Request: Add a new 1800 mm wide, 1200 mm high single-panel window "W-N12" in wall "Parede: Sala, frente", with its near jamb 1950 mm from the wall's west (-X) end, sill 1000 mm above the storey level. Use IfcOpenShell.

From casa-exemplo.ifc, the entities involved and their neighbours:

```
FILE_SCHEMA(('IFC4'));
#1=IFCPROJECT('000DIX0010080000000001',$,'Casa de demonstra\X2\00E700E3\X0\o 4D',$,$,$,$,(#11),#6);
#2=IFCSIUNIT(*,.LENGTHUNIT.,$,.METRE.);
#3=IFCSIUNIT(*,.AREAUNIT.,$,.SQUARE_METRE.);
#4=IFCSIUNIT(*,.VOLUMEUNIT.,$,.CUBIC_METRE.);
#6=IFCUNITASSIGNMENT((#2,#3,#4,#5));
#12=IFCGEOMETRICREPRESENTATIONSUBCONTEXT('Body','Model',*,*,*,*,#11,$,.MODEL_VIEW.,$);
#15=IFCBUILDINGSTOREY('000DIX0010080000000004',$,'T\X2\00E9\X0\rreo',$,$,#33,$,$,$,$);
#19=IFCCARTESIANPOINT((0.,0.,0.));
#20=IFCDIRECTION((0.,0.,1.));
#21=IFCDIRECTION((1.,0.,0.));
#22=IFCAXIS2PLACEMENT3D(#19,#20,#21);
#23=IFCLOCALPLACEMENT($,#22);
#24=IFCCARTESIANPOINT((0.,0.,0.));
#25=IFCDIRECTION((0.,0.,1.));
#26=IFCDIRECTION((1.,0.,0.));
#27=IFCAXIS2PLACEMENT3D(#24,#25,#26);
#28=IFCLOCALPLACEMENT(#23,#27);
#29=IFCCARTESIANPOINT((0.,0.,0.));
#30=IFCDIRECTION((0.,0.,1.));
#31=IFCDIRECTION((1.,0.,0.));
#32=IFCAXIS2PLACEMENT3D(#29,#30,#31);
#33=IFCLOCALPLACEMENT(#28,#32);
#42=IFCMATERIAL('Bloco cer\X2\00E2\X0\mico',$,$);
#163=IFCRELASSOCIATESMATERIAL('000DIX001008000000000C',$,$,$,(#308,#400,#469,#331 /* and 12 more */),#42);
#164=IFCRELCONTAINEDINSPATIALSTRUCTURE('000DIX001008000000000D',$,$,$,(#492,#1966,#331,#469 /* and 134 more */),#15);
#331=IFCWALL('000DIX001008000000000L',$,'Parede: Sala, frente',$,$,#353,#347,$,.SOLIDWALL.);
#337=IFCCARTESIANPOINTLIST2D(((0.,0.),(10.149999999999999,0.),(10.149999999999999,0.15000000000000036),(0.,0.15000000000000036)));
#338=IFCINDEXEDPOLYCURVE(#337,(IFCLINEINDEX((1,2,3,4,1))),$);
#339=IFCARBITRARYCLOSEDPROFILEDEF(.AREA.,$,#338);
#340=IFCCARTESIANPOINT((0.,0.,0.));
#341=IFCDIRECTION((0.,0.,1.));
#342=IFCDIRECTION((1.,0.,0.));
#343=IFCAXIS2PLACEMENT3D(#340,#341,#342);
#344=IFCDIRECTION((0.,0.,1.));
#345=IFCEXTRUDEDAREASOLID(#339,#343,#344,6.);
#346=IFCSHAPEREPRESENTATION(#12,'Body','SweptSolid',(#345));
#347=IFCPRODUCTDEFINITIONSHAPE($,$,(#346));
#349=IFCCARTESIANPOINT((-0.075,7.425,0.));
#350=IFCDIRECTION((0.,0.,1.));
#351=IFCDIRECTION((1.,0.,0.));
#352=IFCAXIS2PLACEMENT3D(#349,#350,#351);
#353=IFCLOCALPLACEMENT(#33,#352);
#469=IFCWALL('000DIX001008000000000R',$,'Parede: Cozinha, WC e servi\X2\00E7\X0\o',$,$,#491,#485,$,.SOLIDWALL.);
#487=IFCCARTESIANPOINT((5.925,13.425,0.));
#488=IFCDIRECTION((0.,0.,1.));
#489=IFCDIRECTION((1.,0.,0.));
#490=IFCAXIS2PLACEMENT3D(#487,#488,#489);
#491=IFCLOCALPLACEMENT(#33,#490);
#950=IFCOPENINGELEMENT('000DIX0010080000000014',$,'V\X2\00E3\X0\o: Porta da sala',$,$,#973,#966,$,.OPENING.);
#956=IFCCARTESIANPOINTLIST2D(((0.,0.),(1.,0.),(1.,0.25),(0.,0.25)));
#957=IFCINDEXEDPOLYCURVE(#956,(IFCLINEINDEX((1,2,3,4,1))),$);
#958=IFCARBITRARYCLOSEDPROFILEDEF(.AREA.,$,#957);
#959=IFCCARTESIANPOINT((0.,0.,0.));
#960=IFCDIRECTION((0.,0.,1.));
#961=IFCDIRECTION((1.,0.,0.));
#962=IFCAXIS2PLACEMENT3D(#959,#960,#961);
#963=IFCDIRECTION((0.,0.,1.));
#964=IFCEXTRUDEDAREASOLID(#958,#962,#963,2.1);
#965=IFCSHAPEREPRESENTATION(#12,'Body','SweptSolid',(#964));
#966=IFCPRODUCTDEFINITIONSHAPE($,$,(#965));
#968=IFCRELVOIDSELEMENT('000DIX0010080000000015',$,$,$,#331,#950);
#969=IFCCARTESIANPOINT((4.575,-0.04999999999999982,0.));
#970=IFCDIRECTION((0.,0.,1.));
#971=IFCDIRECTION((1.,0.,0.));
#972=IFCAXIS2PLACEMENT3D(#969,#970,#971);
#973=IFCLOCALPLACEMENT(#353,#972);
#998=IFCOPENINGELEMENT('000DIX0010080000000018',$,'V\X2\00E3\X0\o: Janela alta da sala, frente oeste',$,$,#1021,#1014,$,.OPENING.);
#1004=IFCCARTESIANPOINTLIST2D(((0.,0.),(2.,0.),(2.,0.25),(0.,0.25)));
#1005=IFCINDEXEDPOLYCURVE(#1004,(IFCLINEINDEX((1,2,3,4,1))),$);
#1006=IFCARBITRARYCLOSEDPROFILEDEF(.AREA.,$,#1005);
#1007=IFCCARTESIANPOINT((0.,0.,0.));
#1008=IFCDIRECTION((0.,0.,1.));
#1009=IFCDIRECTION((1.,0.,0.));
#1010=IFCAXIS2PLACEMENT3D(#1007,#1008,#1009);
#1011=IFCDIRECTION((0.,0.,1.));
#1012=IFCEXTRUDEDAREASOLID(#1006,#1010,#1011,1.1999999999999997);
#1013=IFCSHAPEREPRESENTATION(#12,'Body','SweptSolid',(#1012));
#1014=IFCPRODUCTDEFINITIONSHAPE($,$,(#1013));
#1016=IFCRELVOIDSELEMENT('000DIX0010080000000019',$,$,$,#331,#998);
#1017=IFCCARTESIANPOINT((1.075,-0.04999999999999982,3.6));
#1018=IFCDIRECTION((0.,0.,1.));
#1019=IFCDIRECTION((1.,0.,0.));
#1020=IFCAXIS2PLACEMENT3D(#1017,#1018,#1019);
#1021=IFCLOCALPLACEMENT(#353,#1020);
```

```python
import numpy as np
import ifcopenshell
import ifcopenshell.api.feature
import ifcopenshell.api.geometry
import ifcopenshell.api.root
import ifcopenshell.api.spatial
import ifcopenshell.geom
import ifcopenshell.util.element
import ifcopenshell.util.placement
import ifcopenshell.util.representation
import ifcopenshell.util.shape
import ifcopenshell.util.unit

model = ifcopenshell.open("casa-exemplo.ifc")
unit_scale = ifcopenshell.util.unit.calculate_unit_scale(model)
settings = ifcopenshell.geom.settings()


def volume(element):
    """Net volume in cubic metres, openings subtracted."""
    shape = ifcopenshell.geom.create_shape(settings, element)
    return ifcopenshell.util.shape.get_volume(shape.geometry)


wall = model.by_guid("000DIX001008000000000L")
storey = ifcopenshell.util.element.get_container(wall, ifc_class="IfcBuildingStorey")
context = ifcopenshell.util.representation.get_context(model, "Model", "Body", "MODEL_VIEW")
before = volume(wall)

width, height, from_end, sill = 1.8, 1.2, 1.95, 1  # metres

# The wall runs along its own X axis, and the end named is its -X end.
wall_shape = ifcopenshell.geom.create_shape(settings, wall)
x, y, z = ifcopenshell.util.shape.get_vertices(wall_shape.geometry).T
start = x.min() + from_end
face, thickness = float(y.min()), float(y.max() - y.min())
wall_matrix = ifcopenshell.util.placement.get_local_placement(wall.ObjectPlacement)
level = ifcopenshell.util.placement.get_local_placement(storey.ObjectPlacement)[2, 3]


def in_wall(x, y):
    """Placement at x, y metres in the wall's axes, at sill height."""
    matrix = wall_matrix.copy()
    matrix[:, 3] = wall_matrix @ np.array([x / unit_scale, y / unit_scale, 0.0, 1.0])
    matrix[2, 3] = level + sill / unit_scale
    return matrix


# Opening: a box that overshoots both wall faces by 50 mm.
opening = ifcopenshell.api.root.create_entity(model, ifc_class="IfcOpeningElement", predefined_type="OPENING")
box = ifcopenshell.api.geometry.add_wall_representation(
    model, context=context, length=width, height=height, thickness=thickness + 0.1
)
ifcopenshell.api.geometry.assign_representation(model, product=opening, representation=box)
ifcopenshell.api.geometry.edit_object_placement(model, product=opening, matrix=in_wall(start, face - 0.05), is_si=False)
ifcopenshell.api.feature.add_feature(model, feature=opening, element=wall)

window = ifcopenshell.api.root.create_entity(model, ifc_class="IfcWindow", name="W-N12", predefined_type="WINDOW")
window.OverallWidth, window.OverallHeight = width / unit_scale, height / unit_scale
window.PartitioningType = "SINGLE_PANEL"
body = ifcopenshell.api.geometry.add_window_representation(
    model,
    context=context,
    overall_width=window.OverallWidth,
    overall_height=window.OverallHeight,
    partition_type="SINGLE_PANEL",
)
ifcopenshell.api.geometry.assign_representation(model, product=window, representation=body)
ifcopenshell.api.spatial.assign_container(model, products=[window], relating_structure=storey)
ifcopenshell.api.feature.add_filling(model, opening=opening, element=window)

# Centre the window in the wall's thickness.
ifcopenshell.api.geometry.edit_object_placement(model, product=window, matrix=in_wall(start, face), is_si=False)
window_shape = ifcopenshell.geom.create_shape(settings, window)
depth = ifcopenshell.util.shape.get_vertices(window_shape.geometry)[:, 1]
offset = face + thickness / 2 - (depth.min() + depth.max()) / 2
ifcopenshell.api.geometry.edit_object_placement(model, product=window, matrix=in_wall(start, offset), is_si=False)

after = volume(wall)

print(f"wall volume {before:.3f} -> {after:.3f} m3")

model.write("casa-exemplo_edited.ifc")
```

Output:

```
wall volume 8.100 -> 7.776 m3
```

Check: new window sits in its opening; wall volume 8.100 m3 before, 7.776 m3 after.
